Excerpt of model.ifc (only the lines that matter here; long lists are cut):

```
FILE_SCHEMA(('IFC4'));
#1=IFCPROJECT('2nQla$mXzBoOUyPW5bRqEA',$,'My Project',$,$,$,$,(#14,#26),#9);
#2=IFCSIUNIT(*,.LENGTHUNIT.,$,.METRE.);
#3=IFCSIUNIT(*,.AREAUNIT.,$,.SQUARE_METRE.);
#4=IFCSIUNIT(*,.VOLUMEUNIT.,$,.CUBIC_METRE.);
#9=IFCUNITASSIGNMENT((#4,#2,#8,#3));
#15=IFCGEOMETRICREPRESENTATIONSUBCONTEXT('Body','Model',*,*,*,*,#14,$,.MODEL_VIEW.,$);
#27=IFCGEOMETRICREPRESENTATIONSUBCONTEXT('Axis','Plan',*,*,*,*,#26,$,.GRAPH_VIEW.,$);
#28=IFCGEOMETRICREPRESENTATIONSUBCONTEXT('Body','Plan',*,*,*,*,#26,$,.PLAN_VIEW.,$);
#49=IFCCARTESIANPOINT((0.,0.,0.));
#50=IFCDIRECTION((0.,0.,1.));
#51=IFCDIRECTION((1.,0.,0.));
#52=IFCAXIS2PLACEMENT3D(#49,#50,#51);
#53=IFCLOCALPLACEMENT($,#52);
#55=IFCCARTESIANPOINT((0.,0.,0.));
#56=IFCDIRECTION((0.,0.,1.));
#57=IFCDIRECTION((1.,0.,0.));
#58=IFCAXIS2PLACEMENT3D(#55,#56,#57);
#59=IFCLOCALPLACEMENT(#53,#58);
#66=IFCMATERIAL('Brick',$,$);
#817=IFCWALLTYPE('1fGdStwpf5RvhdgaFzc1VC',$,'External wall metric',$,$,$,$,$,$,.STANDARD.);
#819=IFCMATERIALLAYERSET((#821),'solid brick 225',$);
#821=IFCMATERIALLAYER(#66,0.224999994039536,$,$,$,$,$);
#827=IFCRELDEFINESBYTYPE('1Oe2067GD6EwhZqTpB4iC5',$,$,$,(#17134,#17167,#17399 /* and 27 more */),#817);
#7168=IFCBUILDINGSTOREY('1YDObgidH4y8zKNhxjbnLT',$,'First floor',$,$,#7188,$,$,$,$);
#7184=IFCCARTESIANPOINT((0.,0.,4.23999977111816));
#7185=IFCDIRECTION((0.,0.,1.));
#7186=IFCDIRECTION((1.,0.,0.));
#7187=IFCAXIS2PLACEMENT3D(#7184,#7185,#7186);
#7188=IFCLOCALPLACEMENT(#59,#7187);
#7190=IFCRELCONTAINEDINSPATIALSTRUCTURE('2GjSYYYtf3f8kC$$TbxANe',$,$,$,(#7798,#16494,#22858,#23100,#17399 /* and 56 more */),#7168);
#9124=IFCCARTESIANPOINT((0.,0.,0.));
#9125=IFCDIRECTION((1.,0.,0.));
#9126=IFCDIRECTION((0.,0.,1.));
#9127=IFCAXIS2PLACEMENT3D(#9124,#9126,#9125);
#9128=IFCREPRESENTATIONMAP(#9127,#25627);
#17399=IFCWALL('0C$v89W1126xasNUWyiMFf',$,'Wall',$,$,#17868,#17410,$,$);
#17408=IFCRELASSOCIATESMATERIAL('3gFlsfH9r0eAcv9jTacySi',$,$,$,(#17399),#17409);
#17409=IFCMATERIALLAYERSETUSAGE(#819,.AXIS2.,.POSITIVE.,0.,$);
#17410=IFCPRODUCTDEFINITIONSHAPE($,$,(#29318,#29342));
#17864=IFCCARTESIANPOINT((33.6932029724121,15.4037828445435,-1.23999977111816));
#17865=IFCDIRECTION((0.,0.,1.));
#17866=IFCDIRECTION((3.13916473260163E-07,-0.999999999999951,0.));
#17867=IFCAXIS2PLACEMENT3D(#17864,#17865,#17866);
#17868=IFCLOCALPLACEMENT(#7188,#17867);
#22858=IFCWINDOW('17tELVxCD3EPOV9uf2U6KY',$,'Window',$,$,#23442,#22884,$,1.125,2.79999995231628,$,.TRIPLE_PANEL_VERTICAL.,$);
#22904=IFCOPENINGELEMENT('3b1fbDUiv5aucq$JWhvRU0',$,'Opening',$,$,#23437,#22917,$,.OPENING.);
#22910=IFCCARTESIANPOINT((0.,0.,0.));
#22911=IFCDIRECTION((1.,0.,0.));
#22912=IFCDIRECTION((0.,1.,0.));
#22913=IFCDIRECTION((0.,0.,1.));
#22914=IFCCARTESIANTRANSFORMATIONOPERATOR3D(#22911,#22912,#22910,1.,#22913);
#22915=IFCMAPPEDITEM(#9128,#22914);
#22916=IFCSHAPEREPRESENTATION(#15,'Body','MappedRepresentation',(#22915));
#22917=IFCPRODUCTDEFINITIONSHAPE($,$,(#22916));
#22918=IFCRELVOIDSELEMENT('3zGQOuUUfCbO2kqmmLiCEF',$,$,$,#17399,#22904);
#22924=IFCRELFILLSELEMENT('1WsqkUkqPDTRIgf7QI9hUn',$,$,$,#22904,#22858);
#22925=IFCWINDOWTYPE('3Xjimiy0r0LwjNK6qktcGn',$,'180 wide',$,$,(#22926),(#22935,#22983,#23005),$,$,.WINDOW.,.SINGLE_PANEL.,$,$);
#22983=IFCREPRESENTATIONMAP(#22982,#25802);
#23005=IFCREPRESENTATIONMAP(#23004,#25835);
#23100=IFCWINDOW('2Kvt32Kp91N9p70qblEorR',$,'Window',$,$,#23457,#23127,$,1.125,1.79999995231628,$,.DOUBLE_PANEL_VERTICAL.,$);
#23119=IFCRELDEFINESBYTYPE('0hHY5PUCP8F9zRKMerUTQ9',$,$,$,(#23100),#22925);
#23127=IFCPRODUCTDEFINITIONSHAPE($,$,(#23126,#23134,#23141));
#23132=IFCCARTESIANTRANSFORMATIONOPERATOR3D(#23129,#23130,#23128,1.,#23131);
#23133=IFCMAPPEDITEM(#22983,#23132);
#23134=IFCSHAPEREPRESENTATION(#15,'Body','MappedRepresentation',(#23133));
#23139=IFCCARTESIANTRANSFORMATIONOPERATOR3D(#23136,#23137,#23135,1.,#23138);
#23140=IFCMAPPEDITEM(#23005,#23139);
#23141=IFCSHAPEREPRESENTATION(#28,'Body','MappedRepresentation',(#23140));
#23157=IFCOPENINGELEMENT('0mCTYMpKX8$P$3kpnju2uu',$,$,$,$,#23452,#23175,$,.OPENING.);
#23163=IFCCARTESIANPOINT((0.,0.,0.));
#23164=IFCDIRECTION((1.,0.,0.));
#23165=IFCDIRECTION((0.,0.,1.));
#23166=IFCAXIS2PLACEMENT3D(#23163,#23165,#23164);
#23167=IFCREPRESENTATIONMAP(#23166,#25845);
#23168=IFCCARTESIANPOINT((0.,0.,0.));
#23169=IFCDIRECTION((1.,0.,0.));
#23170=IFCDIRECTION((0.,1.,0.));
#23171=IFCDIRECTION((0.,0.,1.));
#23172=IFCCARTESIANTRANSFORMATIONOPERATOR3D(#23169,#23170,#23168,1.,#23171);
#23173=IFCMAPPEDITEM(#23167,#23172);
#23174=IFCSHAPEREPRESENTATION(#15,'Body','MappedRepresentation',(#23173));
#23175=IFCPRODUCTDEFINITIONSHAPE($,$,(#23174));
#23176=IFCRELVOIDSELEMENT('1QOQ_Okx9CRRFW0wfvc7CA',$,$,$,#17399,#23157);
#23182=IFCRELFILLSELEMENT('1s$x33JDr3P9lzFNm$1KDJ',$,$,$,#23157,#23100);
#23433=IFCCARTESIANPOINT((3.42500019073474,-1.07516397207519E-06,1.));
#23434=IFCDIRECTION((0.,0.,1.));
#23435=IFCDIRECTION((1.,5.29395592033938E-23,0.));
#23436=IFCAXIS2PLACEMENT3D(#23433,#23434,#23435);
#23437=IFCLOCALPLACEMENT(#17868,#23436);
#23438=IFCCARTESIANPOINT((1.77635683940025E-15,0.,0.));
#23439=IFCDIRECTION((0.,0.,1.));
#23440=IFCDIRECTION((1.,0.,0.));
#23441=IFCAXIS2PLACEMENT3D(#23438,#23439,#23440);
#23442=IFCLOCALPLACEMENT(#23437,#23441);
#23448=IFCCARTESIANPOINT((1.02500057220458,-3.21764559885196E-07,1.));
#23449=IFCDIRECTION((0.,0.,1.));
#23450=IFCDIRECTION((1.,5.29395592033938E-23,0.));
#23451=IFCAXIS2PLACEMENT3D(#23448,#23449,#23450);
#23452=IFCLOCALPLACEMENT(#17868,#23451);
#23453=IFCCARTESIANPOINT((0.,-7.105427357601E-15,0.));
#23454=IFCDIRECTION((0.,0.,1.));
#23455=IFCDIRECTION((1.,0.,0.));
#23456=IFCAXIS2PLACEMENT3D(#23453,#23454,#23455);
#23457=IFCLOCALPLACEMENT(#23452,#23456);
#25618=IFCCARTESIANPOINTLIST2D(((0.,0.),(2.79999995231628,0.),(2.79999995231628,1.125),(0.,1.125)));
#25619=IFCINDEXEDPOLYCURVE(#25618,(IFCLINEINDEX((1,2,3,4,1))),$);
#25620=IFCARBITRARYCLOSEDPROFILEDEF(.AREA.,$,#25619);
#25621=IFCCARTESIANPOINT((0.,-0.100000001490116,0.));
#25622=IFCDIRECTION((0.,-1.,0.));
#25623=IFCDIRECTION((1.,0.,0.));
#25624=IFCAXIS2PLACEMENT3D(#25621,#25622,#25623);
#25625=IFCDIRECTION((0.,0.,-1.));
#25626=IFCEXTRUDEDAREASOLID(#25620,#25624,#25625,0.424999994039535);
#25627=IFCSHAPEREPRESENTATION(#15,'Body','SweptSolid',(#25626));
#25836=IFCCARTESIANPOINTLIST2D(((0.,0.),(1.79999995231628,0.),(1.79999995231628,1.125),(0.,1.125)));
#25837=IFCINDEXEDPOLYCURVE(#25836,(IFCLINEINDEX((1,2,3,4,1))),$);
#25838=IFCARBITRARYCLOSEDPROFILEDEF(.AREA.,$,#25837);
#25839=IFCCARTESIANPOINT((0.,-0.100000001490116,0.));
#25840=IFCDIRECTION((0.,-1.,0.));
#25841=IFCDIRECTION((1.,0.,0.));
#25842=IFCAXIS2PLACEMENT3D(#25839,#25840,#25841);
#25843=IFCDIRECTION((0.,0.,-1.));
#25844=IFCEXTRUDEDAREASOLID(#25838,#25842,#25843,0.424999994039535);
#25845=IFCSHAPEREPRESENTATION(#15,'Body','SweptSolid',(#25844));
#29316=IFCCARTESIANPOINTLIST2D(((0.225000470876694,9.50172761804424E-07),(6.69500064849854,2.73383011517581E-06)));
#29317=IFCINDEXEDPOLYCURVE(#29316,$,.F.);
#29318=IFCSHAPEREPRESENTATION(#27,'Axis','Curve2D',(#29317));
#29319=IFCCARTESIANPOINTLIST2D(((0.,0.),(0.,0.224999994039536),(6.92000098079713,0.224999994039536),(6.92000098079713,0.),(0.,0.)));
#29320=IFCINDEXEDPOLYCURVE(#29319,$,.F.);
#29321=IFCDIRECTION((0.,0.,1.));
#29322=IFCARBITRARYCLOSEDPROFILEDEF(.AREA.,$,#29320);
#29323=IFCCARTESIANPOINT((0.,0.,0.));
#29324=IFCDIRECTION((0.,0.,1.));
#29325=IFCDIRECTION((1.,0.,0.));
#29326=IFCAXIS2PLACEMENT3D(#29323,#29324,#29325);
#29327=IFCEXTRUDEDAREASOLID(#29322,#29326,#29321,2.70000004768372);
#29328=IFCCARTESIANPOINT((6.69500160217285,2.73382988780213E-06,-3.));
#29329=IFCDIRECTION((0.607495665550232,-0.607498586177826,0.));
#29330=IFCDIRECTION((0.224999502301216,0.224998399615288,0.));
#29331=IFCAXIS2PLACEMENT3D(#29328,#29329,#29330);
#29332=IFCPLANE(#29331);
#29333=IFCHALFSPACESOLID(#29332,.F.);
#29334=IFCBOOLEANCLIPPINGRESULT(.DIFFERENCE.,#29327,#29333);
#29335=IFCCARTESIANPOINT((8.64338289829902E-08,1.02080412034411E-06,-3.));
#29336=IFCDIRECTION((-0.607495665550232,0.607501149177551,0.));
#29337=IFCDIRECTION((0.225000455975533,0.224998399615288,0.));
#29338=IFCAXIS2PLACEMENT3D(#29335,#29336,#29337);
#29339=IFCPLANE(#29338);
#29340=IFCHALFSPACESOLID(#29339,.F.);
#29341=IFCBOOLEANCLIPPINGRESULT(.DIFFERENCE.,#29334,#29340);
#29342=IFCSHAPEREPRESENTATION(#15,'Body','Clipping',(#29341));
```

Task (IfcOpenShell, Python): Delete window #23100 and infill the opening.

```python
import ifcopenshell
import ifcopenshell.api.feature
import ifcopenshell.api.root
import ifcopenshell.geom
import ifcopenshell.util.shape

model = ifcopenshell.open("model.ifc")
settings = ifcopenshell.geom.settings()


def volume(element):
    """Net volume in cubic metres, openings subtracted."""
    shape = ifcopenshell.geom.create_shape(settings, element)
    return ifcopenshell.util.shape.get_volume(shape.geometry)


window = model.by_guid("2Kvt32Kp91N9p70qblEorR")
opening = window.FillsVoids[0].RelatingOpeningElement
wall = opening.VoidsElements[0].RelatingBuildingElement
before = volume(wall)

ifcopenshell.api.root.remove_product(model, product=window)
ifcopenshell.api.feature.remove_feature(model, feature=opening)

after = volume(wall)

print(f"wall volume {before:.3f} -> {after:.3f} m3")

model.write("model_rev.ifc")
```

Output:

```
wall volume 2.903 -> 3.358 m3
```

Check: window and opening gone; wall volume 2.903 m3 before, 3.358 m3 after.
